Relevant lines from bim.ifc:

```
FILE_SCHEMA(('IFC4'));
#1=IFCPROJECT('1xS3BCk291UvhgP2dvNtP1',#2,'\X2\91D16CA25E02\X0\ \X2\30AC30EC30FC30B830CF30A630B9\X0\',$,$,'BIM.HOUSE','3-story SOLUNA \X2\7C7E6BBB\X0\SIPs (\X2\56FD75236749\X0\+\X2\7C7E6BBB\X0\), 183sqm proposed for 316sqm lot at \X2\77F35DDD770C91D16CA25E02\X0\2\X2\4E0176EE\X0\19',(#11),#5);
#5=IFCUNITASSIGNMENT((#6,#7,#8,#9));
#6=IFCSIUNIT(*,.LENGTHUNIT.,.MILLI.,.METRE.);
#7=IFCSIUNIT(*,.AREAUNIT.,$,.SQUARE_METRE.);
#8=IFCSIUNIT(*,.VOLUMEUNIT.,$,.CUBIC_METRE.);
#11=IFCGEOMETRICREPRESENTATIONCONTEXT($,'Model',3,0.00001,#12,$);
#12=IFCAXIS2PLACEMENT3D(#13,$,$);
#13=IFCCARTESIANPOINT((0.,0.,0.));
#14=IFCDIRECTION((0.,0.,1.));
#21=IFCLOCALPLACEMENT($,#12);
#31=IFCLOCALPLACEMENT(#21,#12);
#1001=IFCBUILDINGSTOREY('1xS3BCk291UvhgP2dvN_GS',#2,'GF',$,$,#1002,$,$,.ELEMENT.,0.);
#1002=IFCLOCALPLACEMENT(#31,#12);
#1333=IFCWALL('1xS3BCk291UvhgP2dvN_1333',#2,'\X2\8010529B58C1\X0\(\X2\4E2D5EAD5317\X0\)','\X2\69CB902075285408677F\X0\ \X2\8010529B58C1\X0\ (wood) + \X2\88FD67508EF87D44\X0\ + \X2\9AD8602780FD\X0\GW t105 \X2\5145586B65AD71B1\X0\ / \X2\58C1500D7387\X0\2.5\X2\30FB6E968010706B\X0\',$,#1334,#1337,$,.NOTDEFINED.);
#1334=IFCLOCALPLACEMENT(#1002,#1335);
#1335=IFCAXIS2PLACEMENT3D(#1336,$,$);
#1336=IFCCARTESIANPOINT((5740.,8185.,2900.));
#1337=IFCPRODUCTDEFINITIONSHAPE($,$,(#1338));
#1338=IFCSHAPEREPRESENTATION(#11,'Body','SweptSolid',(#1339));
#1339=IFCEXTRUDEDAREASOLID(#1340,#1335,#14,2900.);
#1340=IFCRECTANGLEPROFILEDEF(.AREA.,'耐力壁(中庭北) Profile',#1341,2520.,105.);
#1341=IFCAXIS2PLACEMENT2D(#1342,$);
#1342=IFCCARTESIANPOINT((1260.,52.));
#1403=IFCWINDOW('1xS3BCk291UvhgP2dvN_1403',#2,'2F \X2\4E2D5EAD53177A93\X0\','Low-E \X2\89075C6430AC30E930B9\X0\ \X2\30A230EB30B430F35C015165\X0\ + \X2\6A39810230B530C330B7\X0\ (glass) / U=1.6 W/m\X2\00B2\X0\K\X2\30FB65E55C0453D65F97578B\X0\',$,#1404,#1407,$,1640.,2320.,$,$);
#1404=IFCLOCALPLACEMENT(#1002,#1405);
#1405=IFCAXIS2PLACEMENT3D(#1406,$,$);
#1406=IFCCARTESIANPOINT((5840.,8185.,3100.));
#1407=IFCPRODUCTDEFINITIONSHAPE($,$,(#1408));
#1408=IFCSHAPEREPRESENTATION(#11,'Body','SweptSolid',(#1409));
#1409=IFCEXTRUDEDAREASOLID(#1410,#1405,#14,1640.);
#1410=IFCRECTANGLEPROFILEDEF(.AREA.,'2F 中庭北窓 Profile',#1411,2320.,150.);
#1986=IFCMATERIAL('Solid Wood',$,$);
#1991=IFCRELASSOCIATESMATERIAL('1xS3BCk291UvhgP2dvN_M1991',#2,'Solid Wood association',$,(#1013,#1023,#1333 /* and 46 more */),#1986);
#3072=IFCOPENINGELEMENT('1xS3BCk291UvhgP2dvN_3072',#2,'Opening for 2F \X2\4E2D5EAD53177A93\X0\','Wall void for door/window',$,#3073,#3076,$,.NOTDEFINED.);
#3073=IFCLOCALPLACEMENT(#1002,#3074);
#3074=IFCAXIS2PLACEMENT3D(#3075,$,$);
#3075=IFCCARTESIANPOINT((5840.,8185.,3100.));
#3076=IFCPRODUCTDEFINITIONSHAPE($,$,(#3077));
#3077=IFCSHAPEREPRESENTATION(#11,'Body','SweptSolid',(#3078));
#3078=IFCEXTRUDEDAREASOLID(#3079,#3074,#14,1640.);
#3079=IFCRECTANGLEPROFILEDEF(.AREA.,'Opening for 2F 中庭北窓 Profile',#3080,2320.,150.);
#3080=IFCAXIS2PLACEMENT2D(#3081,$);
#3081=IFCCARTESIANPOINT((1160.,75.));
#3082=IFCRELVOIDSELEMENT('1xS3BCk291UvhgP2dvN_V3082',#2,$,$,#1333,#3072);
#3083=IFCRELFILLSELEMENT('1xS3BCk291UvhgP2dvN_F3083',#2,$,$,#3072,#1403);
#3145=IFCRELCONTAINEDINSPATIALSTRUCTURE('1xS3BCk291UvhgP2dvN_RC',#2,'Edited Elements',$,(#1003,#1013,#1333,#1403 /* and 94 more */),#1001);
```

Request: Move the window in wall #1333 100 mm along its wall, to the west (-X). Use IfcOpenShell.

```python
import ifcopenshell
import ifcopenshell.api.geometry
import ifcopenshell.util.placement
import ifcopenshell.util.unit

model = ifcopenshell.open("bim.ifc")
unit_scale = ifcopenshell.util.unit.calculate_unit_scale(model)

window = model.by_guid("1xS3BCk291UvhgP2dvN_1403")
opening = window.FillsVoids[0].RelatingOpeningElement
wall = opening.VoidsElements[0].RelatingBuildingElement

wall_matrix = ifcopenshell.util.placement.get_local_placement(wall.ObjectPlacement)
shift = wall_matrix[:3, 0] * -0.1 / unit_scale
before = ifcopenshell.util.placement.get_local_placement(window.ObjectPlacement)[:3, 3].copy()

# The window is not placed relative to its opening, so move both.
for product in (opening, window):
    matrix = ifcopenshell.util.placement.get_local_placement(product.ObjectPlacement)
    matrix[:3, 3] += shift
    ifcopenshell.api.geometry.edit_object_placement(model, product=product, matrix=matrix, is_si=False)

after = ifcopenshell.util.placement.get_local_placement(window.ObjectPlacement)[:3, 3]
print("window moved by", (after - before).round(3) + 0.0)

model.write("bim-out.ifc")
```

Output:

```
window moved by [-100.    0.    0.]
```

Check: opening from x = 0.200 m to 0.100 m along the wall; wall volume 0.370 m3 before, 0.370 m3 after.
